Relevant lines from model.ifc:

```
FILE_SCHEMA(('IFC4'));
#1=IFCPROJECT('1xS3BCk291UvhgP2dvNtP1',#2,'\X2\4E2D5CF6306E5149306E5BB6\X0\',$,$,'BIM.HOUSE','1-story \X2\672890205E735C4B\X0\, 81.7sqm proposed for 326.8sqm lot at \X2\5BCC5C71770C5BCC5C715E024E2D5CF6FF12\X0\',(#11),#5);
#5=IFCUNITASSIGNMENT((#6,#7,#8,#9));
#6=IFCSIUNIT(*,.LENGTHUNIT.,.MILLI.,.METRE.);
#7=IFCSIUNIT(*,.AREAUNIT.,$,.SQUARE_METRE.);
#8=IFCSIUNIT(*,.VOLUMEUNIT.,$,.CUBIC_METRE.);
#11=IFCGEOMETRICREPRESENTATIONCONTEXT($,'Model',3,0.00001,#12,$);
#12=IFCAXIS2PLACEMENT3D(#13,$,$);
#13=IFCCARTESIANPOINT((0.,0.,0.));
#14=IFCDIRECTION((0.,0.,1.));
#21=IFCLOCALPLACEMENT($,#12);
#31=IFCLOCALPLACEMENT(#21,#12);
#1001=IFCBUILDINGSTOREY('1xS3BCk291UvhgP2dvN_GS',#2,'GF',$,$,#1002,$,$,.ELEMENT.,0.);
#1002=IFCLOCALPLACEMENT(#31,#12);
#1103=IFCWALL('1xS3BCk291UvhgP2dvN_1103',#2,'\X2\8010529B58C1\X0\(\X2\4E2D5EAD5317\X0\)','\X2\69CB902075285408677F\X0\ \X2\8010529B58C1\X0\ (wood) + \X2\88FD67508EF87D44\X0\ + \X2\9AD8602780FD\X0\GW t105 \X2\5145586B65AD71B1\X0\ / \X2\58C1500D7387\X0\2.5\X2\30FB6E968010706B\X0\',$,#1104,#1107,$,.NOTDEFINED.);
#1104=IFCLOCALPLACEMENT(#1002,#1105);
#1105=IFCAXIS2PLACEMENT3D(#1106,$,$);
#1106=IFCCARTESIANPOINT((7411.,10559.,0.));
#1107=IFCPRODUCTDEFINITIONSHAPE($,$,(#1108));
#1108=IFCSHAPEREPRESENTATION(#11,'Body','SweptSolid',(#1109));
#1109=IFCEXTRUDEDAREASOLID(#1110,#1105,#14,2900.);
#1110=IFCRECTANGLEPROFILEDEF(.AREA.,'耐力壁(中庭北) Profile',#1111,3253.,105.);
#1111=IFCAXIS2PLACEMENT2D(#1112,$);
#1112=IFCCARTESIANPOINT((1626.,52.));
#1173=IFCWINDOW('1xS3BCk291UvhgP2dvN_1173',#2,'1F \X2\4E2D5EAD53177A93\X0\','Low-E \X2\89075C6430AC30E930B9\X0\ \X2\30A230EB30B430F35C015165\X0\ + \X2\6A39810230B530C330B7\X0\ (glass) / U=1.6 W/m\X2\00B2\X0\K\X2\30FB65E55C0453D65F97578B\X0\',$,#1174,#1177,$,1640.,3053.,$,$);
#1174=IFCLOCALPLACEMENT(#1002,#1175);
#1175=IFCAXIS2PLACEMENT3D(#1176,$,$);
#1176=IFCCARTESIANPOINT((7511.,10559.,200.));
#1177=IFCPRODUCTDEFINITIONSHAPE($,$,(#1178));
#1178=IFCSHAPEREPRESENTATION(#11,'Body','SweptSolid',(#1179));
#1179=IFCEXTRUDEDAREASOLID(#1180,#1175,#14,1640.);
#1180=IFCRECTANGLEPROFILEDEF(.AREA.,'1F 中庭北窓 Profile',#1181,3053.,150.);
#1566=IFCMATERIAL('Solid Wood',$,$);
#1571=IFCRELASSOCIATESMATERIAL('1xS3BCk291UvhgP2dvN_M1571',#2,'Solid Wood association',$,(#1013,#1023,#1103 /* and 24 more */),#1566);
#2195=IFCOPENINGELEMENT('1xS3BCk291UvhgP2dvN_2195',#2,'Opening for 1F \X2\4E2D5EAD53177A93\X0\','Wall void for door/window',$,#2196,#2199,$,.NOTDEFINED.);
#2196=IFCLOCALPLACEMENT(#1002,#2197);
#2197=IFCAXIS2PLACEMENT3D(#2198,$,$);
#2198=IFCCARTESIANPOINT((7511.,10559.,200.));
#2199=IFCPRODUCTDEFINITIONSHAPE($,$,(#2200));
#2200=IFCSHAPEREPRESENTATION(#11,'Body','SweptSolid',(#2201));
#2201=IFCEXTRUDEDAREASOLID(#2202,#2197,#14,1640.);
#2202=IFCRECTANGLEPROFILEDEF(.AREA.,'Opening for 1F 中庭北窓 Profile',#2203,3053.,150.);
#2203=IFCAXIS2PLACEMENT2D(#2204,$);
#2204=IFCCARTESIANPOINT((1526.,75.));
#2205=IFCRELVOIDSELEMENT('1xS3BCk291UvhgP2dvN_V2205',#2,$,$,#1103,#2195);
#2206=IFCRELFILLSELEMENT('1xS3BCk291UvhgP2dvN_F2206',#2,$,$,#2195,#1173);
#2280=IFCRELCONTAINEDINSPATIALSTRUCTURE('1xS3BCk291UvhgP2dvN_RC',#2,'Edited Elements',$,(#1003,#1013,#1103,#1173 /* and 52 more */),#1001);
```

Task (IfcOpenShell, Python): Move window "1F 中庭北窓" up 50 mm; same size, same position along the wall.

```python
import numpy as np
import ifcopenshell
import ifcopenshell.api.geometry
import ifcopenshell.util.placement
import ifcopenshell.util.unit

model = ifcopenshell.open("model.ifc")
unit_scale = ifcopenshell.util.unit.calculate_unit_scale(model)

window = model.by_id(1173)
opening = window.FillsVoids[0].RelatingOpeningElement
dz = 0.05 / unit_scale

shift = np.array([0.0, 0.0, dz])
# The window is not placed relative to its opening, so move both.
for product in (opening, window):
    matrix = ifcopenshell.util.placement.get_local_placement(product.ObjectPlacement)
    matrix[:3, 3] += shift
    ifcopenshell.api.geometry.edit_object_placement(model, product=product, matrix=matrix, is_si=False)

print(f"moved by {dz * unit_scale:+.3f} m")

model.write("model_updated.ifc")
```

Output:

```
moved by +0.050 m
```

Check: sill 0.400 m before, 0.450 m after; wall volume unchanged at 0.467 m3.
